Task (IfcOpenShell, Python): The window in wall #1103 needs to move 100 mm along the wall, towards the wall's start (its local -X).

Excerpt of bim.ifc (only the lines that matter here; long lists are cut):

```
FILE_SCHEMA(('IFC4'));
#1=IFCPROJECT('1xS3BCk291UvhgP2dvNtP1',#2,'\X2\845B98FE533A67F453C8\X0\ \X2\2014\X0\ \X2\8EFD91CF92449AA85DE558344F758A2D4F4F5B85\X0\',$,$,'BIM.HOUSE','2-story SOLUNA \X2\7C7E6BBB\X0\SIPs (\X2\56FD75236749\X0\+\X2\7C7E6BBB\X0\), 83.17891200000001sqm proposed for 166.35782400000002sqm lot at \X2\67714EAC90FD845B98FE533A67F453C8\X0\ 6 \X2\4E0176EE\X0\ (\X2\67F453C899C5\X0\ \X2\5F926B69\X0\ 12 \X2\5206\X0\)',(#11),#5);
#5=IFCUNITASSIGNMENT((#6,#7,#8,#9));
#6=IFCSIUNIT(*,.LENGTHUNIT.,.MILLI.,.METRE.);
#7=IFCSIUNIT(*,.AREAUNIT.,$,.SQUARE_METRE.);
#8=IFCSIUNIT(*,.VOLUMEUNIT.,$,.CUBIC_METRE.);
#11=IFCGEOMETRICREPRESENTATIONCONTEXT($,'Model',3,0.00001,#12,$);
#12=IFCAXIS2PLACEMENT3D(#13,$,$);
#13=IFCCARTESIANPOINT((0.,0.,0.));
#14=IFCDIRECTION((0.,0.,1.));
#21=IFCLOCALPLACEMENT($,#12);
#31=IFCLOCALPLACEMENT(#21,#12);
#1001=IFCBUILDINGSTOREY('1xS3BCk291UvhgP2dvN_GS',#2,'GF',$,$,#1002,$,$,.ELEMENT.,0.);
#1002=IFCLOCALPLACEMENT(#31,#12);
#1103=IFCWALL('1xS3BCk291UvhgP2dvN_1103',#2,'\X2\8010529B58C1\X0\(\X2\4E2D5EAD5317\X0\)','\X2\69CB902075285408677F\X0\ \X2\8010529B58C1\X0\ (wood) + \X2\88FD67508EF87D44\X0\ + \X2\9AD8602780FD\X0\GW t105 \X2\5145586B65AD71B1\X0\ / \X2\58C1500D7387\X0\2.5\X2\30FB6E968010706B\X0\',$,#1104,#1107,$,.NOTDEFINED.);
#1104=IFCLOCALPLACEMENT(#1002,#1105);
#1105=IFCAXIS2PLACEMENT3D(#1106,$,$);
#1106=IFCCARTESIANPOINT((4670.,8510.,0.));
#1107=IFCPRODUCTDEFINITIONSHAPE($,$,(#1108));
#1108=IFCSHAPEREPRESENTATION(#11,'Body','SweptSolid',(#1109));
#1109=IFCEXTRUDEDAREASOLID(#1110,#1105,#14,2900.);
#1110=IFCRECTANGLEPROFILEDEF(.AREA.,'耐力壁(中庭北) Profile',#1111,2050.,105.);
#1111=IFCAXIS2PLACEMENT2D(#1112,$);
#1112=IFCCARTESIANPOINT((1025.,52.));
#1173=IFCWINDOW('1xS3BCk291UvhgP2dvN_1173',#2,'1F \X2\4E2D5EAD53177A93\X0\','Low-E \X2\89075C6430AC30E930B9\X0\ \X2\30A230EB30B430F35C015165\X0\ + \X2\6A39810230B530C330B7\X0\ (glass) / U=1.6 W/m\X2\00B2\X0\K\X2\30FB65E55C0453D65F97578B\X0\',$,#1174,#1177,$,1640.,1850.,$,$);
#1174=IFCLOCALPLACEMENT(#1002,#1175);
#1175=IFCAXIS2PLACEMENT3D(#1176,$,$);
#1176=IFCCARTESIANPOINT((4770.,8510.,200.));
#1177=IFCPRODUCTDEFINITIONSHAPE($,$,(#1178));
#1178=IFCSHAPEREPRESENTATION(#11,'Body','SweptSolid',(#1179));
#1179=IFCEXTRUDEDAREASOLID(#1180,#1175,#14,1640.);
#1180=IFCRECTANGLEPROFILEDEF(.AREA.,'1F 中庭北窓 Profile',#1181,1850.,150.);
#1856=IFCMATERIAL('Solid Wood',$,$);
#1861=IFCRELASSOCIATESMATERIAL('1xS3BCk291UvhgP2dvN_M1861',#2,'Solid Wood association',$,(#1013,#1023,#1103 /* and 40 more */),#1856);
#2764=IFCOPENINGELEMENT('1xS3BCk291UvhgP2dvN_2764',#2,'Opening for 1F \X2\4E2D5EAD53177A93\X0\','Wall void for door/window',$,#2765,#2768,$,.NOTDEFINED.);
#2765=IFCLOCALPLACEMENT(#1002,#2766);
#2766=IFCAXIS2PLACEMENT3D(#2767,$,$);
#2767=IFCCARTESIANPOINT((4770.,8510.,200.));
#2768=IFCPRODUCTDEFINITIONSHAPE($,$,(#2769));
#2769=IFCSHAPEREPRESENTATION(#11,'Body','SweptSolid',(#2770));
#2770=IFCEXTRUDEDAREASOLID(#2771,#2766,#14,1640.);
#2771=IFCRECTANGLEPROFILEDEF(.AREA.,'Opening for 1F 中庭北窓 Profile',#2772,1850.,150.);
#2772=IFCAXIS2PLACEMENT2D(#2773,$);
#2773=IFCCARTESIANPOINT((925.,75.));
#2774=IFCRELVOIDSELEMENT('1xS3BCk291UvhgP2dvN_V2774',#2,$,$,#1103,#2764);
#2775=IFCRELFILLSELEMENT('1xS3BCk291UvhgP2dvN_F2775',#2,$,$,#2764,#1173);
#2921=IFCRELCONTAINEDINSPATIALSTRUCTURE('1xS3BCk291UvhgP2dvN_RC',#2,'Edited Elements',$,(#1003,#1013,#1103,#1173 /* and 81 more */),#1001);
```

```python
import ifcopenshell
import ifcopenshell.api.geometry
import ifcopenshell.util.placement

model = ifcopenshell.open("bim.ifc")

window = model.by_guid("1xS3BCk291UvhgP2dvN_1173")
opening = window.FillsVoids[0].RelatingOpeningElement
wall = opening.VoidsElements[0].RelatingBuildingElement

wall_matrix = ifcopenshell.util.placement.get_local_placement(wall.ObjectPlacement)
shift = wall_matrix[:3, 0] * -100.0
before = ifcopenshell.util.placement.get_local_placement(window.ObjectPlacement)[:3, 3].copy()

# The window is not placed relative to its opening, so move both.
for product in (opening, window):
    matrix = ifcopenshell.util.placement.get_local_placement(product.ObjectPlacement)
    matrix[:3, 3] += shift
    ifcopenshell.api.geometry.edit_object_placement(model, product=product, matrix=matrix, is_si=False)

after = ifcopenshell.util.placement.get_local_placement(window.ObjectPlacement)[:3, 3]
print("window moved by", (after - before).round(3) + 0.0)

model.write("bim_edited.ifc")
```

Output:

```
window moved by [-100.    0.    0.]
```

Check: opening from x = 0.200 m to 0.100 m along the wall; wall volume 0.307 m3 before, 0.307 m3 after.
